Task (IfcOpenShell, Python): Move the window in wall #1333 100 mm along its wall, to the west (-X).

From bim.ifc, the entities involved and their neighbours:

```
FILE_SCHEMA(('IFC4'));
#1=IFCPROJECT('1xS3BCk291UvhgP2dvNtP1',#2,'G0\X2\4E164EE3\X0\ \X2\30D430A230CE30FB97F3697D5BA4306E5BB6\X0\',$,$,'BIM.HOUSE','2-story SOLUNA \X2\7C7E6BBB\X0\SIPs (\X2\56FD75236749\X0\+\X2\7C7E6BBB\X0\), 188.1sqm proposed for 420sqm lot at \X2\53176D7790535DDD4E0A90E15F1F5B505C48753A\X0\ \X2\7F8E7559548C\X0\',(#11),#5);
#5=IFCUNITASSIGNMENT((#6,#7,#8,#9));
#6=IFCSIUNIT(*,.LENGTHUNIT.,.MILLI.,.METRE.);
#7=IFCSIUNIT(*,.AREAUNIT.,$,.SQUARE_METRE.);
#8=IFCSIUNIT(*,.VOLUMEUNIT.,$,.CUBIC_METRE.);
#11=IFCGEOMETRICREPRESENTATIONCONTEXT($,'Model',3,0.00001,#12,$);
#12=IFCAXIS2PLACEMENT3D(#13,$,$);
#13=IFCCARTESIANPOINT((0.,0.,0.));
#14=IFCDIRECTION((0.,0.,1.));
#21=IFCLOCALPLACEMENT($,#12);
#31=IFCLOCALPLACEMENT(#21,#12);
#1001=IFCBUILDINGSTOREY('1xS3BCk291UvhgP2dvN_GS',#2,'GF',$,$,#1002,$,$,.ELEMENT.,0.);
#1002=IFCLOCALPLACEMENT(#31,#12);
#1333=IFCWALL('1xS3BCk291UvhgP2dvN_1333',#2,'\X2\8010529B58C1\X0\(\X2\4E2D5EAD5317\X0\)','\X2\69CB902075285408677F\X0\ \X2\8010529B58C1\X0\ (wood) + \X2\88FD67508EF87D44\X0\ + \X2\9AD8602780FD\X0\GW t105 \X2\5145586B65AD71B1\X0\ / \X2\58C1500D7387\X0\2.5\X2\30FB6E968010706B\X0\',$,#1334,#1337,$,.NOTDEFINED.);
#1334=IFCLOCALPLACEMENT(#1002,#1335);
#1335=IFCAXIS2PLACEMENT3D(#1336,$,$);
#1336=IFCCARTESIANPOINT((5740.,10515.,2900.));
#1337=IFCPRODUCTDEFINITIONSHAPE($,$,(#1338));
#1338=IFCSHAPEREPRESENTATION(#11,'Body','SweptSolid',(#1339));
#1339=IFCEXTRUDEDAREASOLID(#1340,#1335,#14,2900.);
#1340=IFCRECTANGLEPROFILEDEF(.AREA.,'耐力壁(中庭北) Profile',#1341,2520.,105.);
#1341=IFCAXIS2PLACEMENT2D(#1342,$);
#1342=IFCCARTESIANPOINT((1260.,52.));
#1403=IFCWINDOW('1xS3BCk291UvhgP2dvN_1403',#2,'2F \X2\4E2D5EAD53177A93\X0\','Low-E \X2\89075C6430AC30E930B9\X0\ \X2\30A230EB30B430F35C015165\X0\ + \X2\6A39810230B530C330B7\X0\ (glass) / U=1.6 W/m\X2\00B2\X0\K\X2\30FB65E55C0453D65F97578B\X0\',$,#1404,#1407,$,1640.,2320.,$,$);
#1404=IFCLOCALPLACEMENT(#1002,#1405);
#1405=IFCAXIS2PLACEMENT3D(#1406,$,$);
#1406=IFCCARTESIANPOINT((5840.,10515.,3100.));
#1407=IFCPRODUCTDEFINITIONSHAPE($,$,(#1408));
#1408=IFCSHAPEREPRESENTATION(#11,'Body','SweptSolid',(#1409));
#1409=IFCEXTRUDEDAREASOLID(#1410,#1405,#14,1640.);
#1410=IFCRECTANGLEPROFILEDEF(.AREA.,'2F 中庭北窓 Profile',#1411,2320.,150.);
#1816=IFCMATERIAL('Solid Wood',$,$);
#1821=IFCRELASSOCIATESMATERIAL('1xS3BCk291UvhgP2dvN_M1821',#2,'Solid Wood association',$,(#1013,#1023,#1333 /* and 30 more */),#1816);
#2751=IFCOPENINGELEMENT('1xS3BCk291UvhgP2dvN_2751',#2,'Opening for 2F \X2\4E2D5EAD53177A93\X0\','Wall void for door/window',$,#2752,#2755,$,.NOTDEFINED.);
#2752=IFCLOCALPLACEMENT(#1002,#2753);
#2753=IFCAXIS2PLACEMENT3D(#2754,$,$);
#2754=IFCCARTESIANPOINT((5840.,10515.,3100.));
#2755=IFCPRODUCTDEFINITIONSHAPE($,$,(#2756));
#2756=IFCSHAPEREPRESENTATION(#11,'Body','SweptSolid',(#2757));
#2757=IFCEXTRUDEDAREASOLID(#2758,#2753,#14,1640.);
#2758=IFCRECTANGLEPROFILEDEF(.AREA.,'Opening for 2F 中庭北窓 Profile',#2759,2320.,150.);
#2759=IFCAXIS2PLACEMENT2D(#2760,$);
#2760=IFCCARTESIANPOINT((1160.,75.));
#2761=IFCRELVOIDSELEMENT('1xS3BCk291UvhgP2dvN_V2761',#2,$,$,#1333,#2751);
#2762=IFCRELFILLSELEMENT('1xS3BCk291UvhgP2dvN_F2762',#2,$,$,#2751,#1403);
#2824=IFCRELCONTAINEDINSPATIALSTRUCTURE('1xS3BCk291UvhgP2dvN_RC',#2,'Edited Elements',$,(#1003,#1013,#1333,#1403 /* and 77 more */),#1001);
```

```python
import ifcopenshell
import ifcopenshell.api.geometry
import ifcopenshell.util.placement

model = ifcopenshell.open("bim.ifc")

window = model.by_guid("1xS3BCk291UvhgP2dvN_1403")
opening = window.FillsVoids[0].RelatingOpeningElement
wall = opening.VoidsElements[0].RelatingBuildingElement

wall_matrix = ifcopenshell.util.placement.get_local_placement(wall.ObjectPlacement)
shift = wall_matrix[:3, 0] * -100.0
before = ifcopenshell.util.placement.get_local_placement(window.ObjectPlacement)[:3, 3].copy()

# The window is not placed relative to its opening, so move both.
for product in (opening, window):
    matrix = ifcopenshell.util.placement.get_local_placement(product.ObjectPlacement)
    matrix[:3, 3] += shift
    ifcopenshell.api.geometry.edit_object_placement(model, product=product, matrix=matrix, is_si=False)

after = ifcopenshell.util.placement.get_local_placement(window.ObjectPlacement)[:3, 3]
print("window moved by", (after - before).round(3) + 0.0)

model.write("bim_edited.ifc")
```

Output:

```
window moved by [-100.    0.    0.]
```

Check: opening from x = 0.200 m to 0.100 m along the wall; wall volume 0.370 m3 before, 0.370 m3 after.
